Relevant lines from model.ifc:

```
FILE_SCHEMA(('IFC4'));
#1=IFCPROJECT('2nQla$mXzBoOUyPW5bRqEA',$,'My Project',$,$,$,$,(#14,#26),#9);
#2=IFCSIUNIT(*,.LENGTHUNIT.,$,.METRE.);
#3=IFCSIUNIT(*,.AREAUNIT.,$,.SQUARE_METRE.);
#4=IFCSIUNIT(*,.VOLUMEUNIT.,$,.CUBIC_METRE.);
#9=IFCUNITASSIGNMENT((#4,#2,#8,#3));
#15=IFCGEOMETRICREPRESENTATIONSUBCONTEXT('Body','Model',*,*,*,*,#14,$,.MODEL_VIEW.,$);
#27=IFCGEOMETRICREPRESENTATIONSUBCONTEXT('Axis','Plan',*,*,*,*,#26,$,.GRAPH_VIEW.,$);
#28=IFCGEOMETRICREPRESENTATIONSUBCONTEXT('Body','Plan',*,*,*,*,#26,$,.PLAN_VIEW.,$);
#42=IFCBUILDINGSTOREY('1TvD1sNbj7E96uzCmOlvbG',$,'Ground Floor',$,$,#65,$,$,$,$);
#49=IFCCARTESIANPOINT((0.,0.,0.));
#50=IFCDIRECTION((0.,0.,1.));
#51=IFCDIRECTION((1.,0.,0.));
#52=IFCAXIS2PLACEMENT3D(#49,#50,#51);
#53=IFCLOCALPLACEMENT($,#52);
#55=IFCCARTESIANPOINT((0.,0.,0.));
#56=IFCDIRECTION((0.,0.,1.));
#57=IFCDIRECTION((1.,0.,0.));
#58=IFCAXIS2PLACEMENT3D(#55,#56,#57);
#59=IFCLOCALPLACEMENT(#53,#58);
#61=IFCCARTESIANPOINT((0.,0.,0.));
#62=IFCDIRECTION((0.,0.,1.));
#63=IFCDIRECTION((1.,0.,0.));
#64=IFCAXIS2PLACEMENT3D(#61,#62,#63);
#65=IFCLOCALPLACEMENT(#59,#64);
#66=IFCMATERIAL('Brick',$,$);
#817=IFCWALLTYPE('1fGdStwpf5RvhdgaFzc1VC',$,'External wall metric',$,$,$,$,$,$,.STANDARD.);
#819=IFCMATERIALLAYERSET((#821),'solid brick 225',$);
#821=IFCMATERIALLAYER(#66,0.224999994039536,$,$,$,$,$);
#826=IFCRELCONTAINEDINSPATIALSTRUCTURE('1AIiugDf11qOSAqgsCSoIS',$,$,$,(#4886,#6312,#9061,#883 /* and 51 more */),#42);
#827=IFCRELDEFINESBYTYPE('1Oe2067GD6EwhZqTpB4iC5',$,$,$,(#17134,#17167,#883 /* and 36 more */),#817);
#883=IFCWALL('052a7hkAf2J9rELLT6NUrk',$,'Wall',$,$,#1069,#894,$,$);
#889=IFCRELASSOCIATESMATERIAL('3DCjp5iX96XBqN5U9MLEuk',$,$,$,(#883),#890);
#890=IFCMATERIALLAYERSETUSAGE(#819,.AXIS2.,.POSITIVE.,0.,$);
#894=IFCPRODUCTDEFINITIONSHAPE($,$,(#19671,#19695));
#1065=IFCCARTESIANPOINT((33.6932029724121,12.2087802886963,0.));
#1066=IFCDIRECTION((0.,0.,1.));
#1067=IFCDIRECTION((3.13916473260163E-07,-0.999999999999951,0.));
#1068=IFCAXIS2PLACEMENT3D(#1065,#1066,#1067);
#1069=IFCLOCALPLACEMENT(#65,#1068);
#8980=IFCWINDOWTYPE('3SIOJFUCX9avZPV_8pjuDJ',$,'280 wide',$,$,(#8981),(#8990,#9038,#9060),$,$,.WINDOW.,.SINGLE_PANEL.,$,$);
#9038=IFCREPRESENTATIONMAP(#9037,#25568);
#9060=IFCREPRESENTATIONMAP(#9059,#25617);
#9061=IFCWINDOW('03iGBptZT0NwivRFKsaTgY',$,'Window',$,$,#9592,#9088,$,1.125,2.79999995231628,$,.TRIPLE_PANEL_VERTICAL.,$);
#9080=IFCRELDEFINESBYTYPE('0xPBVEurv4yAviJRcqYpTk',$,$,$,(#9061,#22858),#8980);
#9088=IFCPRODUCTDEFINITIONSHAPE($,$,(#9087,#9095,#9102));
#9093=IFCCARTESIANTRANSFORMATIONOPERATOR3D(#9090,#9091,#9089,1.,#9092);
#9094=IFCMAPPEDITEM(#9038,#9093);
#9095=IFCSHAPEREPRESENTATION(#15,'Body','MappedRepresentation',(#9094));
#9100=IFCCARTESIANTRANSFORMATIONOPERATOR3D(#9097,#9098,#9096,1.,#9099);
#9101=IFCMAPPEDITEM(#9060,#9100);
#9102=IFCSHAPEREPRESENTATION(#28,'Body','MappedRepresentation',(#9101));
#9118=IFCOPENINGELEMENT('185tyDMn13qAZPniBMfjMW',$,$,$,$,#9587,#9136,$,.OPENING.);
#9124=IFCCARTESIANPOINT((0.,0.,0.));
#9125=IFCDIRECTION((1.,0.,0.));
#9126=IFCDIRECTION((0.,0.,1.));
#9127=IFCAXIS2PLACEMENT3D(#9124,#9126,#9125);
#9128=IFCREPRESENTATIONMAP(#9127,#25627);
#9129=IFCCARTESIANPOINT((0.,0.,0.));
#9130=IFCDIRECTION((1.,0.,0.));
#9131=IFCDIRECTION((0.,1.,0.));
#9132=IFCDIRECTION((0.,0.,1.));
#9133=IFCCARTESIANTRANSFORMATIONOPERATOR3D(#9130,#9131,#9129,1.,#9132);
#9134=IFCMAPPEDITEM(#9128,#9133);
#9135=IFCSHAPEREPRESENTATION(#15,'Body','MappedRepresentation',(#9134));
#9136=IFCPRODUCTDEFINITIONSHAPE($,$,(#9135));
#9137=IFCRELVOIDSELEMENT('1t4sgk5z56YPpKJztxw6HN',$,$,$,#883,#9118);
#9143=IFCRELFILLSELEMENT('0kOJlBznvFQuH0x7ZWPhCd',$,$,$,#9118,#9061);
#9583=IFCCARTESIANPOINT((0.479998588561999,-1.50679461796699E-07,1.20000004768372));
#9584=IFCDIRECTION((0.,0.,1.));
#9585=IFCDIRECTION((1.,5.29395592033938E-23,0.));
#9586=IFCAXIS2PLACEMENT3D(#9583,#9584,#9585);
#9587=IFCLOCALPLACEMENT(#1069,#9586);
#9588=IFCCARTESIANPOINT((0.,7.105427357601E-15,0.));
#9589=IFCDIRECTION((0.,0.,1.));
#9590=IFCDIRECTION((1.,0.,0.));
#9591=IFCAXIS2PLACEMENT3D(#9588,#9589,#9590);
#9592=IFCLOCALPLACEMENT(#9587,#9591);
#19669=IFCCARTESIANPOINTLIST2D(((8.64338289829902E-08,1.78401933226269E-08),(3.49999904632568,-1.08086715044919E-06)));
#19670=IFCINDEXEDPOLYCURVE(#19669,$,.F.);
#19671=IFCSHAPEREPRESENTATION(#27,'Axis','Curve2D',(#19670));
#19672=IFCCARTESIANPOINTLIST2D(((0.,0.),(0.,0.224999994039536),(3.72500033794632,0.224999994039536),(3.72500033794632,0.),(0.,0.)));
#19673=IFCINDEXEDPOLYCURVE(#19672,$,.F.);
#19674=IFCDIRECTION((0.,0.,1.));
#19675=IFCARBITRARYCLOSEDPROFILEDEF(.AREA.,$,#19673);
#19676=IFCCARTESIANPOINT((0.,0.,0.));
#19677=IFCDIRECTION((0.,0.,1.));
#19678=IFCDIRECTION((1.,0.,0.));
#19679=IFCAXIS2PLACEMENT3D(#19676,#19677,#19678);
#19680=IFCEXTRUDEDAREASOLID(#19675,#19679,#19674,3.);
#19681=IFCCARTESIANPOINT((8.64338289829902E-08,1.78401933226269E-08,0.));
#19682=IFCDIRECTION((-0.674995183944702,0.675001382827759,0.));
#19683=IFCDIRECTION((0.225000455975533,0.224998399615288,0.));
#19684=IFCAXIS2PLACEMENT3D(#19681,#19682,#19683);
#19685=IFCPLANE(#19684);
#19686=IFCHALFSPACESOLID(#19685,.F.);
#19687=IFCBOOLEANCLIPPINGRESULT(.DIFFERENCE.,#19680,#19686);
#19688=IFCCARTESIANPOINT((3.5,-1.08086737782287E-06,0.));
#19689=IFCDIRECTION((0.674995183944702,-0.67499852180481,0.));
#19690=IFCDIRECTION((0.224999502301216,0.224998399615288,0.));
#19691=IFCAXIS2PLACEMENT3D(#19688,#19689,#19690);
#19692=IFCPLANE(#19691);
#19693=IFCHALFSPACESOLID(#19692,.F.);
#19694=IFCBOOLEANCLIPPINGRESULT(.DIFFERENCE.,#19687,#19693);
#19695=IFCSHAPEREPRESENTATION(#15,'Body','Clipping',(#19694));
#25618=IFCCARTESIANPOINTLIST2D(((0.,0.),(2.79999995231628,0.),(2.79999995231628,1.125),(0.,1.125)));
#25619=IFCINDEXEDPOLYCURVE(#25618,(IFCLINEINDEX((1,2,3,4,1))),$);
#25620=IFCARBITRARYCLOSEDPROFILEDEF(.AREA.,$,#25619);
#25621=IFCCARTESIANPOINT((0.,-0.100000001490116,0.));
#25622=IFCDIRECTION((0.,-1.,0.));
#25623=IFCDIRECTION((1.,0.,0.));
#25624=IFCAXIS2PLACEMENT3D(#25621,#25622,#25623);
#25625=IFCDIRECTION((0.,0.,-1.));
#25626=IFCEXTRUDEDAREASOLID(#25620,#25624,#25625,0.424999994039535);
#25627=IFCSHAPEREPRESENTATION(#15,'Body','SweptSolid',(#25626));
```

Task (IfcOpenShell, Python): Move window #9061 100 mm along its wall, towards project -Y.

```python
import ifcopenshell
import ifcopenshell.api.geometry
import ifcopenshell.util.placement

model = ifcopenshell.open("model.ifc")

window = model.by_guid("03iGBptZT0NwivRFKsaTgY")
opening = window.FillsVoids[0].RelatingOpeningElement
wall = opening.VoidsElements[0].RelatingBuildingElement

wall_matrix = ifcopenshell.util.placement.get_local_placement(wall.ObjectPlacement)
shift = wall_matrix[:3, 0] * 0.1
before = ifcopenshell.util.placement.get_local_placement(window.ObjectPlacement)[:3, 3].copy()

# The window is placed relative to its opening, so it follows when the opening moves.
matrix = ifcopenshell.util.placement.get_local_placement(opening.ObjectPlacement)
matrix[:3, 3] += shift
ifcopenshell.api.geometry.edit_object_placement(
    model, product=opening, matrix=matrix, is_si=False, should_transform_children=True
)

after = ifcopenshell.util.placement.get_local_placement(window.ObjectPlacement)[:3, 3]
print("window moved by", (after - before).round(3) + 0.0)

model.write("model-out.ifc")
```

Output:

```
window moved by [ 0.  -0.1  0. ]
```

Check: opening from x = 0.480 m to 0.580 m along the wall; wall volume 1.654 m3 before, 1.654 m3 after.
